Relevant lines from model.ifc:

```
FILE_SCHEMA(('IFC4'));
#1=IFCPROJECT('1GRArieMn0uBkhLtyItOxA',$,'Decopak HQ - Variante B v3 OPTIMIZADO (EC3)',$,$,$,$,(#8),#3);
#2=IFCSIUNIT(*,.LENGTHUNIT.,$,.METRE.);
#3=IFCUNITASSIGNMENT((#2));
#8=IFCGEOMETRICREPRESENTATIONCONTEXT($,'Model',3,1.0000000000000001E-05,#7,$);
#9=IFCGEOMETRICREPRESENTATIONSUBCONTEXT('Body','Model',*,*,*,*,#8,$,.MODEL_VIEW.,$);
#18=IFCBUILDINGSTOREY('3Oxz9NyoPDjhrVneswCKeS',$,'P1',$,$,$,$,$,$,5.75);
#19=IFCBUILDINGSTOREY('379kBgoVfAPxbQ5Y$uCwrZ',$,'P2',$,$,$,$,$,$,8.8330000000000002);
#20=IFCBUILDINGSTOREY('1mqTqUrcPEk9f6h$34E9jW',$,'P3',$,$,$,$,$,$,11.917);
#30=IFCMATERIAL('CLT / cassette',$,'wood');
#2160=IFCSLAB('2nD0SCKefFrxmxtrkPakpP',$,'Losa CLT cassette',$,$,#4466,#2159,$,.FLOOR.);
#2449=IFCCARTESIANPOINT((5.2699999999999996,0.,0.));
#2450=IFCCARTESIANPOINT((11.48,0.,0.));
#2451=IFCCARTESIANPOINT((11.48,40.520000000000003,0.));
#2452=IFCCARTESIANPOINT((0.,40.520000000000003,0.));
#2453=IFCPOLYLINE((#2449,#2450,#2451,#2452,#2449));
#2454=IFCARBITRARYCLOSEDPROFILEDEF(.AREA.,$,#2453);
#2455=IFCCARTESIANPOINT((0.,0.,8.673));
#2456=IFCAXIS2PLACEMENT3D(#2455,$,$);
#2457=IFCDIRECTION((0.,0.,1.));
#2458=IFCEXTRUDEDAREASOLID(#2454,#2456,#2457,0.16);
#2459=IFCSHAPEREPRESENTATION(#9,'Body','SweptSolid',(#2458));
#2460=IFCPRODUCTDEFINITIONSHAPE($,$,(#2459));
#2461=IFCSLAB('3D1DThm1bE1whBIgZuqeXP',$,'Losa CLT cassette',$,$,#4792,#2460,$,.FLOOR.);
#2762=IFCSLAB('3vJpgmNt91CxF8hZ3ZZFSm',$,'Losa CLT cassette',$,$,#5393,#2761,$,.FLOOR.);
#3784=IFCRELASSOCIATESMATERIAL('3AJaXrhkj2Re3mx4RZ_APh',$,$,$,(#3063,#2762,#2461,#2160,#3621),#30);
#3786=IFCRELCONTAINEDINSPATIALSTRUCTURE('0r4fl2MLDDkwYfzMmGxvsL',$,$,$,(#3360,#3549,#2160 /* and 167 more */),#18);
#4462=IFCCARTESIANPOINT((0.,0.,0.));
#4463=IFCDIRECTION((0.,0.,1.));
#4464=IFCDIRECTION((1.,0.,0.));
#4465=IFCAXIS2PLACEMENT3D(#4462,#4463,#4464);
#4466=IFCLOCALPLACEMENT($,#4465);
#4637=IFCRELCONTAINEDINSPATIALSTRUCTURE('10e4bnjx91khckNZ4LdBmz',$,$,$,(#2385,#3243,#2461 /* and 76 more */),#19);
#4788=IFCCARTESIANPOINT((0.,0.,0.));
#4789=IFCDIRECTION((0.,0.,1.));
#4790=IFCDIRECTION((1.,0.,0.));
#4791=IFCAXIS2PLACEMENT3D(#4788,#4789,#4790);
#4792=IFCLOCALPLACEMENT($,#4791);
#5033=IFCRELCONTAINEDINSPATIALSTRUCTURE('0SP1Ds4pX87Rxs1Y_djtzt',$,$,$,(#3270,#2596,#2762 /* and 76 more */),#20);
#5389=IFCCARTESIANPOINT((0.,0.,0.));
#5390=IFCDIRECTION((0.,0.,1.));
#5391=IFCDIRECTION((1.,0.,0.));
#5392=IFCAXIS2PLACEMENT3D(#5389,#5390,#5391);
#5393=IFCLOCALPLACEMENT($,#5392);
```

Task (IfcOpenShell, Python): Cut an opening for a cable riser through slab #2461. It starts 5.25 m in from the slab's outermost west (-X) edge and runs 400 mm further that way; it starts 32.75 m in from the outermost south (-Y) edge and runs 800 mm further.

```python
import numpy as np
import ifcopenshell
import ifcopenshell.api.feature
import ifcopenshell.api.geometry
import ifcopenshell.api.root
import ifcopenshell.geom
import ifcopenshell.util.placement
import ifcopenshell.util.representation
import ifcopenshell.util.shape
import ifcopenshell.util.unit

model = ifcopenshell.open("model.ifc")
unit_scale = ifcopenshell.util.unit.calculate_unit_scale(model)
settings = ifcopenshell.geom.settings()


def volume(element):
    """Net volume in cubic metres, openings subtracted."""
    shape = ifcopenshell.geom.create_shape(settings, element)
    return ifcopenshell.util.shape.get_volume(shape.geometry)


slab = model.by_guid("3D1DThm1bE1whBIgZuqeXP")
before = volume(slab)

# Extent in the slab's own axes, in metres. The edges named are its -X and -Y sides.
slab_shape = ifcopenshell.geom.create_shape(settings, slab)
vertices = ifcopenshell.util.shape.get_vertices(slab_shape.geometry)
x_min, y_min, bottom = vertices.min(axis=0)
top = vertices[:, 2].max()

opening = ifcopenshell.api.root.create_entity(model, ifc_class="IfcOpeningElement", name="Cable riser opening", predefined_type="OPENING")
context = ifcopenshell.util.representation.get_context(model, "Model", "Body", "MODEL_VIEW")
width, depth = 0.4, 0.8
outline = [(0.0, 0.0), (width, 0.0), (width, depth), (0.0, depth), (0.0, 0.0)]
# Overshoot both faces by 50 mm so the cut is clean.
shape = ifcopenshell.api.geometry.add_slab_representation(
    model, context=context, depth=top - bottom + 0.1, polyline=outline
)
ifcopenshell.api.geometry.assign_representation(model, product=opening, representation=shape)

matrix = ifcopenshell.util.placement.get_local_placement(slab.ObjectPlacement)
matrix[:, 3] = matrix @ np.append(np.array([x_min + 5.25, y_min + 32.75, bottom - 0.05]) / unit_scale, 1.0)
ifcopenshell.api.geometry.edit_object_placement(model, product=opening, matrix=matrix, is_si=False)
ifcopenshell.api.feature.add_feature(model, feature=opening, element=slab)

after = volume(slab)

print(f"slab volume {before:.3f} -> {after:.3f} m3")

model.write("model_rev.ifc")
```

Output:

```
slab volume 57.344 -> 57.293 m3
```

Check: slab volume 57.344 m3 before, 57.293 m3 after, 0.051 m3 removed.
